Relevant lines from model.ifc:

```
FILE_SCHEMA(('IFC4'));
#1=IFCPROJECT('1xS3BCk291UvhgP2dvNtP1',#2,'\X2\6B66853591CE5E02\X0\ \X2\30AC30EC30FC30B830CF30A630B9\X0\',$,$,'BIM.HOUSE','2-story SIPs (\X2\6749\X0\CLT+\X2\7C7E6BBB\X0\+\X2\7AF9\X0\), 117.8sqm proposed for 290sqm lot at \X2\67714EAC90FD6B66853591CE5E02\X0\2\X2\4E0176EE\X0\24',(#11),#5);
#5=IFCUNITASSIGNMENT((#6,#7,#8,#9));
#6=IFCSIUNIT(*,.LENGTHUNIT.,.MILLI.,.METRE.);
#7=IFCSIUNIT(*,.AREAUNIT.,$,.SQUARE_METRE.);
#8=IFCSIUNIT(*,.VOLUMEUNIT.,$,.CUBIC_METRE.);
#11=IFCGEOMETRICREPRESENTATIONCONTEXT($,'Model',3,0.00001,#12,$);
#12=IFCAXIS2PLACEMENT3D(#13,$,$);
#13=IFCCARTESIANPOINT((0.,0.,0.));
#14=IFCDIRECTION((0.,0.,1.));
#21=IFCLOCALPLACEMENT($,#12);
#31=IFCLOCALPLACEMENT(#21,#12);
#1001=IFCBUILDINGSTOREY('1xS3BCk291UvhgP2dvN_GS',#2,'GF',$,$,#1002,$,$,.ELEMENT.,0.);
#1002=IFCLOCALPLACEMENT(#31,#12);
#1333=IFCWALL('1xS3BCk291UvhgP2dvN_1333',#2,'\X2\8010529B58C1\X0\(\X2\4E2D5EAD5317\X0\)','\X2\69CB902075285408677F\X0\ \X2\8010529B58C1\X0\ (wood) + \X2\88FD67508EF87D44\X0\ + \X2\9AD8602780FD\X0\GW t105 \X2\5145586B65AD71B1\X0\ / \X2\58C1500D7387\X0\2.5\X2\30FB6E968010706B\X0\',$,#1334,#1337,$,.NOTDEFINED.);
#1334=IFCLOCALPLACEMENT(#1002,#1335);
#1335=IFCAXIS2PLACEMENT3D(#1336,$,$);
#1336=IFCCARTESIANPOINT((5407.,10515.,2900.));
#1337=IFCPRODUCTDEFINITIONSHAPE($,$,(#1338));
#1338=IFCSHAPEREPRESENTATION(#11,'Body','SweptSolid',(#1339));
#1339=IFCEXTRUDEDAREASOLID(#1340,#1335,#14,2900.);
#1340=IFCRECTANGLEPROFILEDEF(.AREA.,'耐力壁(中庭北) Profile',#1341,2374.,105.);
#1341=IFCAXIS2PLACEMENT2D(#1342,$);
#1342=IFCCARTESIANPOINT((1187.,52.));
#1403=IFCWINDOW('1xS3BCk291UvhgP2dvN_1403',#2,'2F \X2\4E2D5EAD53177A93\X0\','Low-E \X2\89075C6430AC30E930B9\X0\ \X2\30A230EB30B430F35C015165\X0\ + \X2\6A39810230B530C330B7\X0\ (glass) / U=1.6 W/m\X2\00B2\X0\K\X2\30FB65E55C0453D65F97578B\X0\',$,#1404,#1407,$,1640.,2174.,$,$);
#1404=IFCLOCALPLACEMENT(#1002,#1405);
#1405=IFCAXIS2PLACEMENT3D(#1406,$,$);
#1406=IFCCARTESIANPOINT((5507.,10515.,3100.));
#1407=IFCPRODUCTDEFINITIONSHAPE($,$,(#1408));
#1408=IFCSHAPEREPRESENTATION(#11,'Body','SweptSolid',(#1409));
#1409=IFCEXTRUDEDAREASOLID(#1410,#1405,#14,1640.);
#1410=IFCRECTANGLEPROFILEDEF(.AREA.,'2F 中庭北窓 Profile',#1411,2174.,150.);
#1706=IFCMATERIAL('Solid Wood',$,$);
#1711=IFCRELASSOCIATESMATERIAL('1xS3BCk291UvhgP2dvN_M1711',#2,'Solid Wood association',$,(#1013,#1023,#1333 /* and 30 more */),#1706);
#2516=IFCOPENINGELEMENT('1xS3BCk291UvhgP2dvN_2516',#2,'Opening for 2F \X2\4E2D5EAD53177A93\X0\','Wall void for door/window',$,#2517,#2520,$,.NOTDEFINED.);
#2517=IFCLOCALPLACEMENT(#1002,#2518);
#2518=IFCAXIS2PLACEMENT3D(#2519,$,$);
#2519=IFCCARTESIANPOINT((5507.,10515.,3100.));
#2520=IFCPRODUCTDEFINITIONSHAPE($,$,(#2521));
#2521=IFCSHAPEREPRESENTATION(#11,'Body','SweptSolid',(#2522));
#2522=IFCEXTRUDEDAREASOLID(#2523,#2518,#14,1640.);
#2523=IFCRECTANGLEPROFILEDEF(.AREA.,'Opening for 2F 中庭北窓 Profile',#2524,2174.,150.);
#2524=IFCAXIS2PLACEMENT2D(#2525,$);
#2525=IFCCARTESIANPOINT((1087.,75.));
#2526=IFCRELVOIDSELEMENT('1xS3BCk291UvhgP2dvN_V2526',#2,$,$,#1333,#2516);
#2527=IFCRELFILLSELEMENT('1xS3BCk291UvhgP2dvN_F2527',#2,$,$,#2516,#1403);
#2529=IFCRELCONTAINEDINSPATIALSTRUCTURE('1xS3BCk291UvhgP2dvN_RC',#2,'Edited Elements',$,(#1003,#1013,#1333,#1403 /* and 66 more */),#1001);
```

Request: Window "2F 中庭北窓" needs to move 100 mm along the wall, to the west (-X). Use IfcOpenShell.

```python
import ifcopenshell
import ifcopenshell.api.geometry
import ifcopenshell.util.placement

model = ifcopenshell.open("model.ifc")

window = model.by_guid("1xS3BCk291UvhgP2dvN_1403")
opening = window.FillsVoids[0].RelatingOpeningElement
wall = opening.VoidsElements[0].RelatingBuildingElement

wall_matrix = ifcopenshell.util.placement.get_local_placement(wall.ObjectPlacement)
shift = wall_matrix[:3, 0] * -100.0
before = ifcopenshell.util.placement.get_local_placement(window.ObjectPlacement)[:3, 3].copy()

# The window is not placed relative to its opening, so move both.
for product in (opening, window):
    matrix = ifcopenshell.util.placement.get_local_placement(product.ObjectPlacement)
    matrix[:3, 3] += shift
    ifcopenshell.api.geometry.edit_object_placement(model, product=product, matrix=matrix, is_si=False)

after = ifcopenshell.util.placement.get_local_placement(window.ObjectPlacement)[:3, 3]
print("window moved by", (after - before).round(3) + 0.0)

model.write("model_edited.ifc")
```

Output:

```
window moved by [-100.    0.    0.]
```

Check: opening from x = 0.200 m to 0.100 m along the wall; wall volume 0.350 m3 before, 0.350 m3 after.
